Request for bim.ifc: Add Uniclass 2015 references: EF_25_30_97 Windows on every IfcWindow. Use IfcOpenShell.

First a look at what the model holds.

```python
import ifcopenshell

model = ifcopenshell.open("bim.ifc")
print(model.schema)
print("classifications:", [c.Name for c in model.by_type("IfcClassification")])
for ifc_class in ("IfcDoor", "IfcRoof", "IfcStair", "IfcWall", "IfcWindow"):
    print(ifc_class, len(model.by_type(ifc_class)))
```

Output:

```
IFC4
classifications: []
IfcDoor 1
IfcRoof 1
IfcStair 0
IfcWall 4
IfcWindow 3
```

```python
import ifcopenshell
import ifcopenshell.api.classification

model = ifcopenshell.open("bim.ifc")

system = ifcopenshell.api.classification.add_classification(model, classification="Uniclass 2015")

codes = {
    "IfcWindow": ("EF_25_30_97", "Windows"),
}
for ifc_class, (code, name) in codes.items():
    products = model.by_type(ifc_class)
    ifcopenshell.api.classification.add_reference(
        model, products=products, classification=system, identification=code, name=name
    )
    print(code, len(products))

model.write("bim_updated.ifc")
```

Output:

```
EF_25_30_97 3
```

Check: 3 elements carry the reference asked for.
